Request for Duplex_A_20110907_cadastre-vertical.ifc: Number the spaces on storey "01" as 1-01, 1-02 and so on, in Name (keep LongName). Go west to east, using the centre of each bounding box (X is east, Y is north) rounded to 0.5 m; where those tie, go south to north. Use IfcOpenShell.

First a look at what the model holds.

```python
import ifcopenshell
import ifcopenshell.util.element
import ifcopenshell.util.placement

model = ifcopenshell.open("Duplex_A_20110907_cadastre-vertical.ifc")
print(model.schema)
storey = next(s for s in model.by_type("IfcBuildingStorey") if s.Name == "01")
spaces = [e for e in ifcopenshell.util.element.get_decomposition(storey) if e.is_a("IfcSpace")]
for e in sorted(spaces, key=lambda e: e.id()):
    origin = ifcopenshell.util.placement.get_local_placement(e.ObjectPlacement)[:3, 3]
    print(e.id(), e.Name, e.LongName, origin.round(2) + 0.0, sep=" | ")
```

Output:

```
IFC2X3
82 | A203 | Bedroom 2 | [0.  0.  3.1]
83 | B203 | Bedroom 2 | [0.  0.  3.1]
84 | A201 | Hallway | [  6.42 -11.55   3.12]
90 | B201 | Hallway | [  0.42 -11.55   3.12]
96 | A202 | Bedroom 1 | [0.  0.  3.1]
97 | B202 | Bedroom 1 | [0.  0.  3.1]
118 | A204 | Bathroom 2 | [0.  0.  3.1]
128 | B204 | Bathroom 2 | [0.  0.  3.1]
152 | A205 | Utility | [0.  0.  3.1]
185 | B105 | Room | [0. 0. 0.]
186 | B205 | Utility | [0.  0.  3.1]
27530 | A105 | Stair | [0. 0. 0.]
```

```python
import ifcopenshell
import ifcopenshell.geom
import ifcopenshell.util.element
import ifcopenshell.util.shape

model = ifcopenshell.open("Duplex_A_20110907_cadastre-vertical.ifc")
settings = ifcopenshell.geom.settings()
settings.set("use-world-coords", True)


def centre(element):
    shape = ifcopenshell.geom.create_shape(settings, element)
    return ifcopenshell.util.shape.get_bbox_centroid(shape.geometry)


storey = next(s for s in model.by_type("IfcBuildingStorey") if s.Name == "01")
spaces = [e for e in ifcopenshell.util.element.get_decomposition(storey) if e.is_a("IfcSpace")]

# Insertion points can sit at a corner or the storey origin, so sort by the geometry (in metres).
centres = {e: centre(e) for e in spaces}
spaces.sort(key=lambda e: (round(centres[e][0] / 0.5), centres[e][1]))

for i, e in enumerate(spaces, start=1):
    number = f"1-{i:02d}"
    e.Name = number
    print(e.id(), number)

model.write("Duplex_A_20110907_cadastre-vertical_v2.ifc")
```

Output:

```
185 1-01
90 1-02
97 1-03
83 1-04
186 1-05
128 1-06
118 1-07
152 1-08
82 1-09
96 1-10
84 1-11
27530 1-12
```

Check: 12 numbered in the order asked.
